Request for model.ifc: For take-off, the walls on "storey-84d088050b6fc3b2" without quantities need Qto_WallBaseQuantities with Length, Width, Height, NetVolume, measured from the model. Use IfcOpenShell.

First a look at what the model holds.

```python
import ifcopenshell
import ifcopenshell.util.element
import ifcopenshell.util.unit

model = ifcopenshell.open("model.ifc")
print(model.schema)
for unit_type in ("LENGTHUNIT", "AREAUNIT", "VOLUMEUNIT"):
    print(unit_type, ifcopenshell.util.unit.calculate_unit_scale(model, unit_type))
storey = next(s for s in model.by_type("IfcBuildingStorey") if s.Name == "storey-84d088050b6fc3b2")
walls = [e for e in ifcopenshell.util.element.get_decomposition(storey) if e.is_a("IfcWall")]
for e in sorted(walls, key=lambda e: e.id()):
    print(e.id(), e.is_a(), e.Name, list(ifcopenshell.util.element.get_psets(e, qtos_only=True)), sep=" | ")
```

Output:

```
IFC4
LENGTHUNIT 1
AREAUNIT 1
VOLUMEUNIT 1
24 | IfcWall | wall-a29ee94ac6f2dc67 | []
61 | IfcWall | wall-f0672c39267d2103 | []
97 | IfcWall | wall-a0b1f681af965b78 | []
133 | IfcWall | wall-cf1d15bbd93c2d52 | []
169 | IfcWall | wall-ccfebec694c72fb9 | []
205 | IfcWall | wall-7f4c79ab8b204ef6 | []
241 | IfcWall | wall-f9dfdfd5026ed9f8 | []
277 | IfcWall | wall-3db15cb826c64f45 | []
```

```python
import ifcopenshell
import ifcopenshell.api.pset
import ifcopenshell.geom
import ifcopenshell.util.element
import ifcopenshell.util.shape
import ifcopenshell.util.unit

model = ifcopenshell.open("model.ifc")
unit_scale = ifcopenshell.util.unit.calculate_unit_scale(model)
volume_scale = ifcopenshell.util.unit.calculate_unit_scale(model, "VOLUMEUNIT")
settings = ifcopenshell.geom.settings()

storey = next(s for s in model.by_type("IfcBuildingStorey") if s.Name == "storey-84d088050b6fc3b2")
walls = [e for e in ifcopenshell.util.element.get_decomposition(storey) if e.is_a("IfcWall")]

for e in sorted(walls, key=lambda e: e.id()):
    if ifcopenshell.util.element.get_psets(e, qtos_only=True, should_inherit=False):
        continue
    # Geometry comes back in metres, in the element's own axes.
    shape = ifcopenshell.geom.create_shape(settings, e)
    values = {
        "Length": ifcopenshell.util.shape.get_x(shape.geometry) / unit_scale,
        "Width": ifcopenshell.util.shape.get_y(shape.geometry) / unit_scale,
        "Height": ifcopenshell.util.shape.get_z(shape.geometry) / unit_scale,
        "NetVolume": ifcopenshell.util.shape.get_volume(shape.geometry) / volume_scale,
    }
    qto = ifcopenshell.api.pset.add_qto(model, product=e, name="Qto_WallBaseQuantities")
    ifcopenshell.api.pset.edit_qto(model, qto=qto, properties=values)
    print(e.id(), {k: round(v, 3) for k, v in values.items()})

model.write("model_v2.ifc")
```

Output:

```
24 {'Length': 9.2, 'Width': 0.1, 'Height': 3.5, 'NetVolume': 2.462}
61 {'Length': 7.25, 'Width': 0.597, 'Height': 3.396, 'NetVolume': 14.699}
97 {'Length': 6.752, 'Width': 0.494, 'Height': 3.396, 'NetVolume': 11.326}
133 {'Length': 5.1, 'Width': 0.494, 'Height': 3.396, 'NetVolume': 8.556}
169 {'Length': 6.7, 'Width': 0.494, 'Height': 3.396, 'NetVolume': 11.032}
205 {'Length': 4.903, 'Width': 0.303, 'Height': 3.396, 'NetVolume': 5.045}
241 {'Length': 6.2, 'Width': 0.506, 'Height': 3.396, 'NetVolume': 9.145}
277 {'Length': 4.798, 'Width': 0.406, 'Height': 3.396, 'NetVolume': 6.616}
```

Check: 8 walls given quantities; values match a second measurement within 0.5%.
